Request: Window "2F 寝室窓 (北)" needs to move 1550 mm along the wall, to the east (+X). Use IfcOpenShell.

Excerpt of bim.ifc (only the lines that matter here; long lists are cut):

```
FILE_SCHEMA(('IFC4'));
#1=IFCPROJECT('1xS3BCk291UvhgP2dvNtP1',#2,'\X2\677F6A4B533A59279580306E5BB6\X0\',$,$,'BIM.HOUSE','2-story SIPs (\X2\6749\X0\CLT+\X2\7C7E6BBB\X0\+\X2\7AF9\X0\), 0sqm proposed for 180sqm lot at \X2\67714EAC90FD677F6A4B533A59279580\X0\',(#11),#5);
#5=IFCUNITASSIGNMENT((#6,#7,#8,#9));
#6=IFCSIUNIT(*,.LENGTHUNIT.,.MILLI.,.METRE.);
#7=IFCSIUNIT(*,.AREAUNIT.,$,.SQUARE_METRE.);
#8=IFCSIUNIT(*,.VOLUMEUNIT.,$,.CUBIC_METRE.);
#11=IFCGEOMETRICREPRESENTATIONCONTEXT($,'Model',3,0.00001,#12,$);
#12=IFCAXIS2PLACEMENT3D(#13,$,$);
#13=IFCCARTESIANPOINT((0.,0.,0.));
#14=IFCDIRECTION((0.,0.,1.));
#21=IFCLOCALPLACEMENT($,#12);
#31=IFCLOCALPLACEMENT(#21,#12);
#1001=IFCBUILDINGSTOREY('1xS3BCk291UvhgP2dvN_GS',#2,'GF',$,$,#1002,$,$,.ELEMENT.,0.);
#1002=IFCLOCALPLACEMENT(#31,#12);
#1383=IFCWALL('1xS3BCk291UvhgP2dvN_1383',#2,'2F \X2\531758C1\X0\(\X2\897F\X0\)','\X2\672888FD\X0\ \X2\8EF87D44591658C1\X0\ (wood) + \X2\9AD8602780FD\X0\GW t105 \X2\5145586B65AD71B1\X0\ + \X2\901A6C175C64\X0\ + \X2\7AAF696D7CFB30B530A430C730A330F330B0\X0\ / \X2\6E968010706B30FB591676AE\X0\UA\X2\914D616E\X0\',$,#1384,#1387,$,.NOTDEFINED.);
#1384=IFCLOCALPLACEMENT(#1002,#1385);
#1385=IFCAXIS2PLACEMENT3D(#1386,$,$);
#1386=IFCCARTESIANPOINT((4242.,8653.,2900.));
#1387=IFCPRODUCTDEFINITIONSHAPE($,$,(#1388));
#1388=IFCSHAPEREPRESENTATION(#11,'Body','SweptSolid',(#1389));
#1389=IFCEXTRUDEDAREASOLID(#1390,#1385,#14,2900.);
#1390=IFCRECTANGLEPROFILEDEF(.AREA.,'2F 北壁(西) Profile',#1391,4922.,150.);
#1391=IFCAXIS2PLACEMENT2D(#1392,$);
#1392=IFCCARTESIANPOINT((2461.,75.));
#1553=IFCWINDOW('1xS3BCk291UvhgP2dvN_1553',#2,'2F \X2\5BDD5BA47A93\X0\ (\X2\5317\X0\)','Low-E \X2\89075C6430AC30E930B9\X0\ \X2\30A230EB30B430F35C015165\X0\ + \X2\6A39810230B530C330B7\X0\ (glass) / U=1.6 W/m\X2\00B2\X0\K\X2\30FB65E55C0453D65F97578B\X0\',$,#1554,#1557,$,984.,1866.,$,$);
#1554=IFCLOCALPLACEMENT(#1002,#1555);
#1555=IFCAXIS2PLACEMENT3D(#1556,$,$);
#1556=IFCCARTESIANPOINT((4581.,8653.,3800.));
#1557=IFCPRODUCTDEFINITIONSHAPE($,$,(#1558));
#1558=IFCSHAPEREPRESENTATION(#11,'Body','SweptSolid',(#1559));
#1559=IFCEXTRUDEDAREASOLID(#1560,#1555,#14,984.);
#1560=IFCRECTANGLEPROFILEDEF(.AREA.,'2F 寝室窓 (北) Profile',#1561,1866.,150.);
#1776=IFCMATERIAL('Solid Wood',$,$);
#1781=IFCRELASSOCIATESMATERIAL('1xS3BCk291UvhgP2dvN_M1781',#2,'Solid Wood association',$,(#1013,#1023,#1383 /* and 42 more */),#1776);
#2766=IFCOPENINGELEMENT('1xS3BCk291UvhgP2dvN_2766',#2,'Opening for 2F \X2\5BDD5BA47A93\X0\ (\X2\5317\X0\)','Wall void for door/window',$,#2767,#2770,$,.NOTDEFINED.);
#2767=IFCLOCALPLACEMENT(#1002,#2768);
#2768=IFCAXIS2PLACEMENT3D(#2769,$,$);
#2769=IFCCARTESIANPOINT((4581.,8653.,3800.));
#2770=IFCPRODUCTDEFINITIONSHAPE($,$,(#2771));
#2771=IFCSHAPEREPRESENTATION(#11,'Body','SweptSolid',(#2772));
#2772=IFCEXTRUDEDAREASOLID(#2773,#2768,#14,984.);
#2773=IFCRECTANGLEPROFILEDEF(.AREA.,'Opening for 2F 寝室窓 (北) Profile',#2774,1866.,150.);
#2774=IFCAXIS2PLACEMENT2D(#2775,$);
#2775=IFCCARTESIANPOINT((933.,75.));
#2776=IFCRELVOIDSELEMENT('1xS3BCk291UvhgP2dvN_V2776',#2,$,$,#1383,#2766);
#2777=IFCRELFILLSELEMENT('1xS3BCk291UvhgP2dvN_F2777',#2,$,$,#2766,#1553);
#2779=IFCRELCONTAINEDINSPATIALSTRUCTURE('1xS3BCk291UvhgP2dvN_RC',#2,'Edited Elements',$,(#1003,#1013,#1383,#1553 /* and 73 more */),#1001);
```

```python
import ifcopenshell
import ifcopenshell.api.geometry
import ifcopenshell.util.placement
import ifcopenshell.util.unit

model = ifcopenshell.open("bim.ifc")
unit_scale = ifcopenshell.util.unit.calculate_unit_scale(model)

window = model.by_id(1553)
opening = window.FillsVoids[0].RelatingOpeningElement
wall = opening.VoidsElements[0].RelatingBuildingElement

wall_matrix = ifcopenshell.util.placement.get_local_placement(wall.ObjectPlacement)
shift = wall_matrix[:3, 0] * 1.55 / unit_scale
before = ifcopenshell.util.placement.get_local_placement(window.ObjectPlacement)[:3, 3].copy()

# The window is not placed relative to its opening, so move both.
for product in (opening, window):
    matrix = ifcopenshell.util.placement.get_local_placement(product.ObjectPlacement)
    matrix[:3, 3] += shift
    ifcopenshell.api.geometry.edit_object_placement(model, product=product, matrix=matrix, is_si=False)

after = ifcopenshell.util.placement.get_local_placement(window.ObjectPlacement)[:3, 3]
print("window moved by", (after - before).round(3) + 0.0)

model.write("bim_v2.ifc")
```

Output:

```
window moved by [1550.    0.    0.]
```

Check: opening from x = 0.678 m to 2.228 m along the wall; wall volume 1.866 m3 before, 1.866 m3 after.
